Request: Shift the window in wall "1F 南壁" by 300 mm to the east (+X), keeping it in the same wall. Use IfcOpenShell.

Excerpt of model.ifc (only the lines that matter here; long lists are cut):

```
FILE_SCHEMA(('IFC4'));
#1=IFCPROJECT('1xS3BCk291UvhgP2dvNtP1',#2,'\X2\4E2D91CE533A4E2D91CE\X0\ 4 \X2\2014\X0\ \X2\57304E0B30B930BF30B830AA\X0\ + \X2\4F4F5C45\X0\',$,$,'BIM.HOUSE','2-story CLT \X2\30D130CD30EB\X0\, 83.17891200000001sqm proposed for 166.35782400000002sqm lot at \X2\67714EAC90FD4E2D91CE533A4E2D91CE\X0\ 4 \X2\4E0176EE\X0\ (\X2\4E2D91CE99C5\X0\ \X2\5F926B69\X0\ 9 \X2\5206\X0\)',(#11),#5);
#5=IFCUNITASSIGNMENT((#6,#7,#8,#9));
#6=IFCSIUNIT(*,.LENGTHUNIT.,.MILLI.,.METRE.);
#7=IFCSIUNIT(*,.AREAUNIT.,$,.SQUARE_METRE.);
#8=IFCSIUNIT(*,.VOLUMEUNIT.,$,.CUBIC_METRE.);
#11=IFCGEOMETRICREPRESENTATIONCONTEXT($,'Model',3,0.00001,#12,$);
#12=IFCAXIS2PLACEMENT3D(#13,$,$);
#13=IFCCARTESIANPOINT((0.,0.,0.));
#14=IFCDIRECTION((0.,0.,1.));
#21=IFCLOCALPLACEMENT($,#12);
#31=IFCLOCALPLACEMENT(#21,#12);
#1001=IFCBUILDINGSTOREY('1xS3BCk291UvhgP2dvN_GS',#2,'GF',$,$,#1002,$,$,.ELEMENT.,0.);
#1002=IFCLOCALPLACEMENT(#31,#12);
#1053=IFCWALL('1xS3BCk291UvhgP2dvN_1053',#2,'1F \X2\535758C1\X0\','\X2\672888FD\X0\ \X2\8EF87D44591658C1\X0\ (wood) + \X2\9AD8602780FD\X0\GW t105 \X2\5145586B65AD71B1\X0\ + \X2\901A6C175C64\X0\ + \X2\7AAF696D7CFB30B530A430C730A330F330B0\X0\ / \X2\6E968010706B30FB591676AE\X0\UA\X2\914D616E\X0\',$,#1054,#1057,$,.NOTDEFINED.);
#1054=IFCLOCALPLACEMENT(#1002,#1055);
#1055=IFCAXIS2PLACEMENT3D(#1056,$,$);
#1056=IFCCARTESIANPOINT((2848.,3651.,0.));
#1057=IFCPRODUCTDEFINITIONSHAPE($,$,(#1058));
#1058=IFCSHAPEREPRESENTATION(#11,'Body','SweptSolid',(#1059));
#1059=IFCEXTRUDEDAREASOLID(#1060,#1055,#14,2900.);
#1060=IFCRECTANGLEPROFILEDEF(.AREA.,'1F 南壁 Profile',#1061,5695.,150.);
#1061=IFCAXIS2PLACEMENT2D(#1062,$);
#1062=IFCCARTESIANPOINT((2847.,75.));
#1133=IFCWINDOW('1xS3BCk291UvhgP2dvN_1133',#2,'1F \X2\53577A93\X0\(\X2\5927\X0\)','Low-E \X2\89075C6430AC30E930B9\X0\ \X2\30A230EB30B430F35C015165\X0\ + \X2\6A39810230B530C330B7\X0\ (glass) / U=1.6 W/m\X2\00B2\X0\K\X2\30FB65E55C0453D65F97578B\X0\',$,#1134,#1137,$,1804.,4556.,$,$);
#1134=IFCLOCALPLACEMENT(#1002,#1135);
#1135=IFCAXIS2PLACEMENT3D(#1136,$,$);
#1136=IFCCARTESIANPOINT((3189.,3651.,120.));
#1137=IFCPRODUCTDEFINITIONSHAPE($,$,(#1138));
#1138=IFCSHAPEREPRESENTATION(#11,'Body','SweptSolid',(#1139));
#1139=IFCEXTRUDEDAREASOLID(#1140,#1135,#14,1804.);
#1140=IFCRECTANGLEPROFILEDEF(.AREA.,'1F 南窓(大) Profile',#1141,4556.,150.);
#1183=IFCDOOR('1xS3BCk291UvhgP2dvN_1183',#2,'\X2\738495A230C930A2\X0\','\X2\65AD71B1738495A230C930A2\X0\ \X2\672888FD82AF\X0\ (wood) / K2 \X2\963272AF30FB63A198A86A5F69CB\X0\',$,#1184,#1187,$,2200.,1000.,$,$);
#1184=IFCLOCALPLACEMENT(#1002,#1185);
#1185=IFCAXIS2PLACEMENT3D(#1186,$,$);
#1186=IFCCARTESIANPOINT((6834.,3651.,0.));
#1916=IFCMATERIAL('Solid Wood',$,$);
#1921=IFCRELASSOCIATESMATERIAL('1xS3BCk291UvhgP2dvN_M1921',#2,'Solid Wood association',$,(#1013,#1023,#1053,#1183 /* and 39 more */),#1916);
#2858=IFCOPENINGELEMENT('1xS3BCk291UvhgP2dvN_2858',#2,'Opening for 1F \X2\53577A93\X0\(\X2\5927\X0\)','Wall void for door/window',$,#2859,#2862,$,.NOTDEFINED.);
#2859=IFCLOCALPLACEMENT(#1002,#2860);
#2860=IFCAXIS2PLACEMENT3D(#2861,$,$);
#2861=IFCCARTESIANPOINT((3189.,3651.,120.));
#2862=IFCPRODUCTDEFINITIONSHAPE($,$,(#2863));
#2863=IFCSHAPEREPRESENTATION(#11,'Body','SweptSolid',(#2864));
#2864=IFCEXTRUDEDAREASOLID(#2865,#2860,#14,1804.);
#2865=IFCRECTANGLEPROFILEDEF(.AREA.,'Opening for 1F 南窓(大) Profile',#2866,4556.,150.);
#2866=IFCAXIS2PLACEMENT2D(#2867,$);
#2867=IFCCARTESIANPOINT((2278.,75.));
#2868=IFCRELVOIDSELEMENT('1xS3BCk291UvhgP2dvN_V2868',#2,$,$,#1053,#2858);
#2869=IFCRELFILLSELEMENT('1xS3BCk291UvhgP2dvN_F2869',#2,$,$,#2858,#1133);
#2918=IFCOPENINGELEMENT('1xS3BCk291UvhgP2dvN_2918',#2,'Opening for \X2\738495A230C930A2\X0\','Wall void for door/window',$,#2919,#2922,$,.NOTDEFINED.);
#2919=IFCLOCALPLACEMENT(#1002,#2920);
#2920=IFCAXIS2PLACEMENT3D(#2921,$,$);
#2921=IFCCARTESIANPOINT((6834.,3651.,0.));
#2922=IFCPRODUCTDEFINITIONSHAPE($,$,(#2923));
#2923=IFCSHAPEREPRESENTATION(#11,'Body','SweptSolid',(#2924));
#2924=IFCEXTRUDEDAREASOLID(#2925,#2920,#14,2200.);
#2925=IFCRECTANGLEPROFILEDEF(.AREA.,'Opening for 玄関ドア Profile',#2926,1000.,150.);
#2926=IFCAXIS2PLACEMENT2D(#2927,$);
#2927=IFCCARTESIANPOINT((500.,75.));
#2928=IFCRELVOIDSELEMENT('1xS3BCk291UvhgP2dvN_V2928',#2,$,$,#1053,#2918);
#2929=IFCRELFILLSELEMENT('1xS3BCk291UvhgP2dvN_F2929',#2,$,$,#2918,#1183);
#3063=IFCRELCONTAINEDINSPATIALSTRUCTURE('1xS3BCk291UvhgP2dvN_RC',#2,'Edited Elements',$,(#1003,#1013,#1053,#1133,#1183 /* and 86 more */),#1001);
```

```python
import ifcopenshell
import ifcopenshell.api.geometry
import ifcopenshell.util.placement
import ifcopenshell.util.unit

model = ifcopenshell.open("model.ifc")
unit_scale = ifcopenshell.util.unit.calculate_unit_scale(model)

window = model.by_guid("1xS3BCk291UvhgP2dvN_1133")
opening = window.FillsVoids[0].RelatingOpeningElement
wall = opening.VoidsElements[0].RelatingBuildingElement

wall_matrix = ifcopenshell.util.placement.get_local_placement(wall.ObjectPlacement)
shift = wall_matrix[:3, 0] * 0.3 / unit_scale
before = ifcopenshell.util.placement.get_local_placement(window.ObjectPlacement)[:3, 3].copy()

# The window is not placed relative to its opening, so move both.
for product in (opening, window):
    matrix = ifcopenshell.util.placement.get_local_placement(product.ObjectPlacement)
    matrix[:3, 3] += shift
    ifcopenshell.api.geometry.edit_object_placement(model, product=product, matrix=matrix, is_si=False)

after = ifcopenshell.util.placement.get_local_placement(window.ObjectPlacement)[:3, 3]
print("window moved by", (after - before).round(3) + 0.0)

model.write("model_updated.ifc")
```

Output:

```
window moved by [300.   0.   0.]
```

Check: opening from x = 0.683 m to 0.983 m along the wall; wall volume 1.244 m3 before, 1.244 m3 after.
